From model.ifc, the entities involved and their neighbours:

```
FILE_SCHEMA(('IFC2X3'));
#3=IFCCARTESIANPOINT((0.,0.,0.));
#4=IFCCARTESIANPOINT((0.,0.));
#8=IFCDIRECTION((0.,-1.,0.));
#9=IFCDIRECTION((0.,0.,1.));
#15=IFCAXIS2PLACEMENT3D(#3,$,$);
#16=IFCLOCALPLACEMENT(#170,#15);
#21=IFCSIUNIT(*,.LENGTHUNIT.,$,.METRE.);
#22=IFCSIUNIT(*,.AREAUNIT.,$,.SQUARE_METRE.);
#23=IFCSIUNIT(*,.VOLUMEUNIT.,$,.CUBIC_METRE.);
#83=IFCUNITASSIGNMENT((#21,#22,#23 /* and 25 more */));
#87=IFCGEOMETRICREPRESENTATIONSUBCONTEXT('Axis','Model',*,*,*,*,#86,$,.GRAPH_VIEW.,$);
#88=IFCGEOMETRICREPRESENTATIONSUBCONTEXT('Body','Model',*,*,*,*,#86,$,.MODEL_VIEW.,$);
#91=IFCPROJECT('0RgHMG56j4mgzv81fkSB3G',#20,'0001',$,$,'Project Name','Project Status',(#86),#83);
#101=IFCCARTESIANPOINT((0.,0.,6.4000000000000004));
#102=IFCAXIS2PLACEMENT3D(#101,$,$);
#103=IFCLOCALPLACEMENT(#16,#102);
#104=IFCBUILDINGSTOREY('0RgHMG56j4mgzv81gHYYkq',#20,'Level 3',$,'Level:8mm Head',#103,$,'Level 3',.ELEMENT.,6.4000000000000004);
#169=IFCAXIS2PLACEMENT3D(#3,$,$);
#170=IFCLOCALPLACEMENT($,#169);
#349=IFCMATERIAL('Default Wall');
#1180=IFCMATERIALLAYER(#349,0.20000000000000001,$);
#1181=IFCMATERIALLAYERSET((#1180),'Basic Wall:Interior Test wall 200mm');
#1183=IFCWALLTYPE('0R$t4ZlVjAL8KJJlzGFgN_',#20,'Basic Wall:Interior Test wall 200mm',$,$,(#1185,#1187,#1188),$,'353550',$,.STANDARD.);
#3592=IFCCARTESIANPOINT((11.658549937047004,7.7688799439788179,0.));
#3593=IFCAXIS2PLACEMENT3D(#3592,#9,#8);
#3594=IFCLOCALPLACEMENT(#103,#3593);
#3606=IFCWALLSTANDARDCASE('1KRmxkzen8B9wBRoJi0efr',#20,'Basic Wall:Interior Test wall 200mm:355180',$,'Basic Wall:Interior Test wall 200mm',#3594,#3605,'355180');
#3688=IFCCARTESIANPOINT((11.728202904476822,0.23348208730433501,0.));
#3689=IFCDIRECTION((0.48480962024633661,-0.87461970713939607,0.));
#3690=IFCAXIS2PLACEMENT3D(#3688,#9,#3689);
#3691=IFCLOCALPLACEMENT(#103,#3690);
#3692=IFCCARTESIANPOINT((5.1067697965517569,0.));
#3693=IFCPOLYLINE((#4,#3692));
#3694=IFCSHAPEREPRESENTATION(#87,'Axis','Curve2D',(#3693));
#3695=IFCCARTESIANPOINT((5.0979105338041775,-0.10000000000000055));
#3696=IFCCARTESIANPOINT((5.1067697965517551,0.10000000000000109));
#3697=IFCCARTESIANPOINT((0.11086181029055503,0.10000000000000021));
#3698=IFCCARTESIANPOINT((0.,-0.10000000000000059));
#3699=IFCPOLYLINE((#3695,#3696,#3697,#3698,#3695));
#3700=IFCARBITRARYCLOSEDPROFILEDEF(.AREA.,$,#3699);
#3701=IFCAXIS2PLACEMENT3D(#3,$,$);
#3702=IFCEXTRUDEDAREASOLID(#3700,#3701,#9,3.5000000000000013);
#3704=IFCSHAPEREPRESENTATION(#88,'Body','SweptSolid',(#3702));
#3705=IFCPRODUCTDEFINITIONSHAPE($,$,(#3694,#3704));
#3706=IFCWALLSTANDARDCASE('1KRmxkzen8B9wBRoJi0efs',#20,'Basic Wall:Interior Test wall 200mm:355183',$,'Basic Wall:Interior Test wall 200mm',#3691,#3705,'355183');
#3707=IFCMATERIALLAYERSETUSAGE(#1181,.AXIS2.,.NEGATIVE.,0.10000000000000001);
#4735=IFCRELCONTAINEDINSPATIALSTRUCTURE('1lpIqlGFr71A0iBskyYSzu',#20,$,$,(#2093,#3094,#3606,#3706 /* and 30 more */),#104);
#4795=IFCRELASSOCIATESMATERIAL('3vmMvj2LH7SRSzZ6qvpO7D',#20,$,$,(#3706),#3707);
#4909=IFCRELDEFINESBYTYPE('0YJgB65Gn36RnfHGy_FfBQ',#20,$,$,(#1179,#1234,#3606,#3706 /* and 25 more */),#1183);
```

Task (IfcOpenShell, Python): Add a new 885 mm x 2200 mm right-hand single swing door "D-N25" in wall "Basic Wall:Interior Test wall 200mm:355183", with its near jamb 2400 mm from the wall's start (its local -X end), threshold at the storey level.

```python
import numpy as np
import ifcopenshell
import ifcopenshell.api.feature
import ifcopenshell.api.geometry
import ifcopenshell.api.root
import ifcopenshell.api.spatial
import ifcopenshell.api.type
import ifcopenshell.geom
import ifcopenshell.util.element
import ifcopenshell.util.placement
import ifcopenshell.util.representation
import ifcopenshell.util.shape
import ifcopenshell.util.unit

model = ifcopenshell.open("model.ifc")
unit_scale = ifcopenshell.util.unit.calculate_unit_scale(model)
settings = ifcopenshell.geom.settings()


def volume(element):
    """Net volume in cubic metres, openings subtracted."""
    shape = ifcopenshell.geom.create_shape(settings, element)
    return ifcopenshell.util.shape.get_volume(shape.geometry)


wall = model.by_guid("1KRmxkzen8B9wBRoJi0efs")
storey = ifcopenshell.util.element.get_container(wall, ifc_class="IfcBuildingStorey")
context = ifcopenshell.util.representation.get_context(model, "Model", "Body", "MODEL_VIEW")
before = volume(wall)

width, height, from_end, sill = 0.885, 2.2, 2.4, 0.0  # metres

# The wall runs along its own X axis, and the end named is its -X end.
wall_shape = ifcopenshell.geom.create_shape(settings, wall)
x, y, z = ifcopenshell.util.shape.get_vertices(wall_shape.geometry).T
start = x.min() + from_end
face, thickness = float(y.min()), float(y.max() - y.min())
wall_matrix = ifcopenshell.util.placement.get_local_placement(wall.ObjectPlacement)
level = ifcopenshell.util.placement.get_local_placement(storey.ObjectPlacement)[2, 3]


def in_wall(x, y):
    """Placement at x, y metres in the wall's axes, at sill height."""
    matrix = wall_matrix.copy()
    matrix[:, 3] = wall_matrix @ np.array([x / unit_scale, y / unit_scale, 0.0, 1.0])
    matrix[2, 3] = level + sill / unit_scale
    return matrix


# Opening: a box that overshoots both wall faces by 50 mm.
opening = ifcopenshell.api.root.create_entity(model, ifc_class="IfcOpeningElement")
box = ifcopenshell.api.geometry.add_wall_representation(
    model, context=context, length=width, height=height, thickness=thickness + 0.1
)
ifcopenshell.api.geometry.assign_representation(model, product=opening, representation=box)
ifcopenshell.api.geometry.edit_object_placement(model, product=opening, matrix=in_wall(start, face - 0.05), is_si=False)
ifcopenshell.api.feature.add_feature(model, feature=opening, element=wall)

door = ifcopenshell.api.root.create_entity(model, ifc_class="IfcDoor", name="D-N25")
door.OverallWidth, door.OverallHeight = width / unit_scale, height / unit_scale
body = ifcopenshell.api.geometry.add_door_representation(
    model,
    context=context,
    overall_width=door.OverallWidth,
    overall_height=door.OverallHeight,
    operation_type="SINGLE_SWING_RIGHT",
    lining_properties={"LiningDepth": thickness / unit_scale, "ThresholdDepth": thickness / unit_scale},
)
ifcopenshell.api.geometry.assign_representation(model, product=door, representation=body)
ifcopenshell.api.spatial.assign_container(model, products=[door], relating_structure=storey)
fills = ifcopenshell.api.feature.add_filling(model, opening=opening, element=door)
fills.OwnerHistory = door.OwnerHistory  # required in IFC2X3

# IFC2X3 keeps the operation on the door style.
style = ifcopenshell.api.root.create_entity(model, ifc_class="IfcDoorStyle", name="D-N25")
style.OperationType, style.ConstructionType = "SINGLE_SWING_RIGHT", "NOTDEFINED"
style.ParameterTakesPrecedence = style.Sizeable = False
ifcopenshell.api.type.assign_type(model, related_objects=[door], relating_type=style)

# The lining spans the wall, so the door starts at the wall face.
ifcopenshell.api.geometry.edit_object_placement(model, product=door, matrix=in_wall(start, face), is_si=False)

after = volume(wall)

print(f"wall volume {before:.3f} -> {after:.3f} m3")

model.write("model_updated.ifc")
```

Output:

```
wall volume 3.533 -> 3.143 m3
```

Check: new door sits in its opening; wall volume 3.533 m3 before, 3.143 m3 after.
